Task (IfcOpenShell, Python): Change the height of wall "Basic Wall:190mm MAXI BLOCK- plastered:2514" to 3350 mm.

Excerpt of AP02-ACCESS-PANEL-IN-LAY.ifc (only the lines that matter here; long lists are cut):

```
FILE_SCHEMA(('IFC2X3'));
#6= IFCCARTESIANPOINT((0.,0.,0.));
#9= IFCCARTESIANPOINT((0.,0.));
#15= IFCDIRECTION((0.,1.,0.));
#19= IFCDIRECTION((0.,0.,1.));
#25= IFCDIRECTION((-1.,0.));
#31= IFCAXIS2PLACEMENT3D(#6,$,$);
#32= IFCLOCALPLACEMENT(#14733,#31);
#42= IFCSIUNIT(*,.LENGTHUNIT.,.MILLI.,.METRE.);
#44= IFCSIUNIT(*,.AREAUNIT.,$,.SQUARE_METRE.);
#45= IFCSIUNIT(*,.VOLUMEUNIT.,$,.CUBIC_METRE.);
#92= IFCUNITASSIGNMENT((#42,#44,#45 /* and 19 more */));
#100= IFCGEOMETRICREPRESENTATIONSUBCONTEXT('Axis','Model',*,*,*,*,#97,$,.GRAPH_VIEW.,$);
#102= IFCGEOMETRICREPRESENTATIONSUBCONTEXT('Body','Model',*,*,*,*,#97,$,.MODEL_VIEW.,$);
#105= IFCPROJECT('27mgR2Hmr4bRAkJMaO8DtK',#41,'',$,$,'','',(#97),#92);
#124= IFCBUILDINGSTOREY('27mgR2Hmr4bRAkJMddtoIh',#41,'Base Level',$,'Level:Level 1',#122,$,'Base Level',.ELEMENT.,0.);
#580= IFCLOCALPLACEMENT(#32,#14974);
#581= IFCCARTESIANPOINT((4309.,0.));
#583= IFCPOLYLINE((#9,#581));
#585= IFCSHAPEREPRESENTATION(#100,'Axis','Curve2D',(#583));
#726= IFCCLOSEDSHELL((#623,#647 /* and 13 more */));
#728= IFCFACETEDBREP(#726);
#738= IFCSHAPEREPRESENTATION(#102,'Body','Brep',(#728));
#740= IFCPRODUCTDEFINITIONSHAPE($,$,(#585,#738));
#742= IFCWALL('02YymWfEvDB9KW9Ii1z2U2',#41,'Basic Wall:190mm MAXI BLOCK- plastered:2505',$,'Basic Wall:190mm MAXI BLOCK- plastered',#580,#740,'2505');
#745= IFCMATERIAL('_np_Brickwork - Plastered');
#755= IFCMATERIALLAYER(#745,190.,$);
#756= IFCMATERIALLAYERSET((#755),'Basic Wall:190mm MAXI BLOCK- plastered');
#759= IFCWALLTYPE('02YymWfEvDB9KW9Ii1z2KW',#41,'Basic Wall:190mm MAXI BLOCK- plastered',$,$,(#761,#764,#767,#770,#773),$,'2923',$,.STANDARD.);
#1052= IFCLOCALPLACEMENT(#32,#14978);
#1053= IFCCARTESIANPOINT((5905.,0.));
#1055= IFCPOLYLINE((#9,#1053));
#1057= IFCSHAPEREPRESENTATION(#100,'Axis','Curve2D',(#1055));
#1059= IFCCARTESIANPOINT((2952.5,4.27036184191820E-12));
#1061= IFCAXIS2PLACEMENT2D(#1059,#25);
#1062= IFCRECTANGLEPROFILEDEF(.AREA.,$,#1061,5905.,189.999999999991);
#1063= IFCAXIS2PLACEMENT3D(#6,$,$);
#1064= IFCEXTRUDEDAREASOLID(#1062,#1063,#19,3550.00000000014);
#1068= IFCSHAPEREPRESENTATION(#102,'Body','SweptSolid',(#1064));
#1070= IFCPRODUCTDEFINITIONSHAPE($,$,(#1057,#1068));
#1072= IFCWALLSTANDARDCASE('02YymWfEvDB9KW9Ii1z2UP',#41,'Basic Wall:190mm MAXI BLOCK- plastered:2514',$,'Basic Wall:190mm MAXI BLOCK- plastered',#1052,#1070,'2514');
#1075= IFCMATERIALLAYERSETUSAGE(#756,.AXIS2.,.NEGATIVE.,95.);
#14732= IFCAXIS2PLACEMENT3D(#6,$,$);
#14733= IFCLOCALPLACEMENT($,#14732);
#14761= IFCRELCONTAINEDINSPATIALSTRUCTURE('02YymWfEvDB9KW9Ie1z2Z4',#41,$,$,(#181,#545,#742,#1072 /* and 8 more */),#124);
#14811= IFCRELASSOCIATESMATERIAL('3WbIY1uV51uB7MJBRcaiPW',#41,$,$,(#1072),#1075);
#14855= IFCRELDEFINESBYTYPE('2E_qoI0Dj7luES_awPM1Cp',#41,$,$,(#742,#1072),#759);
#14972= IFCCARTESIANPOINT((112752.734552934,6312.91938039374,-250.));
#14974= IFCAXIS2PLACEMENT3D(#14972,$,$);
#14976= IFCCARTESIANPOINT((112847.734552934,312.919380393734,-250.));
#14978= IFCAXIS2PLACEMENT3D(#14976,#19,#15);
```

```python
import ifcopenshell
import ifcopenshell.geom
import ifcopenshell.util.representation
import ifcopenshell.util.shape
import ifcopenshell.util.unit

model = ifcopenshell.open("AP02-ACCESS-PANEL-IN-LAY.ifc")
unit_scale = ifcopenshell.util.unit.calculate_unit_scale(model)
settings = ifcopenshell.geom.settings()


def volume(element):
    """Net volume in cubic metres, openings subtracted."""
    shape = ifcopenshell.geom.create_shape(settings, element)
    return ifcopenshell.util.shape.get_volume(shape.geometry)


wall = model.by_guid("02YymWfEvDB9KW9Ii1z2UP")
before = volume(wall)

body = ifcopenshell.util.representation.get_representation(wall, "Model", "Body")
solid = body.Items[0]
old_height = solid.Depth
solid.Depth = 3.35 / unit_scale
after = volume(wall)

print(f"height {old_height:g} -> {solid.Depth:g}, volume {before:.3f} -> {after:.3f} m3")

model.write("AP02-ACCESS-PANEL-IN-LAY_updated.ifc")
```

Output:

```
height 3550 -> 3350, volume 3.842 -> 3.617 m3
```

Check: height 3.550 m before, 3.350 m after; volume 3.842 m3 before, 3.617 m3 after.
